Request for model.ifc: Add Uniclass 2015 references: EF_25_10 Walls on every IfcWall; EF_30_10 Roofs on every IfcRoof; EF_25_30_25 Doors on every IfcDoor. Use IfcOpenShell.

First a look at what the model holds.

```python
import ifcopenshell

model = ifcopenshell.open("model.ifc")
print(model.schema)
print("classifications:", [c.Name for c in model.by_type("IfcClassification")])
for ifc_class in ("IfcDoor", "IfcRoof", "IfcStair", "IfcWall", "IfcWindow"):
    print(ifc_class, len(model.by_type(ifc_class)))
```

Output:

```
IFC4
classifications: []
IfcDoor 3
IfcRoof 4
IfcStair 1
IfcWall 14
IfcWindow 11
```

```python
import ifcopenshell
import ifcopenshell.api.classification

model = ifcopenshell.open("model.ifc")

system = ifcopenshell.api.classification.add_classification(model, classification="Uniclass 2015")

codes = {
    "IfcWall": ("EF_25_10", "Walls"),
    "IfcRoof": ("EF_30_10", "Roofs"),
    "IfcDoor": ("EF_25_30_25", "Doors"),
}
for ifc_class, (code, name) in codes.items():
    products = model.by_type(ifc_class)
    ifcopenshell.api.classification.add_reference(
        model, products=products, classification=system, identification=code, name=name
    )
    print(code, len(products))

model.write("model-out.ifc")
```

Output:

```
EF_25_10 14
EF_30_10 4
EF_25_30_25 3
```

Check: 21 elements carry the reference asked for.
